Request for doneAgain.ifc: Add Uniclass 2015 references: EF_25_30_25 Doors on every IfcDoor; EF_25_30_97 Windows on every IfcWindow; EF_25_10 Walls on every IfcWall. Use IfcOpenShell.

First a look at what the model holds.

```python
import ifcopenshell

model = ifcopenshell.open("doneAgain.ifc")
print(model.schema)
print("classifications:", [c.Name for c in model.by_type("IfcClassification")])
for ifc_class in ("IfcDoor", "IfcRoof", "IfcStair", "IfcWall", "IfcWindow"):
    print(ifc_class, len(model.by_type(ifc_class)))
```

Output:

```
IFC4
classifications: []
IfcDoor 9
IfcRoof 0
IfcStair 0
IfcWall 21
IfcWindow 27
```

```python
import ifcopenshell
import ifcopenshell.api.classification

model = ifcopenshell.open("doneAgain.ifc")

system = ifcopenshell.api.classification.add_classification(model, classification="Uniclass 2015")

codes = {
    "IfcDoor": ("EF_25_30_25", "Doors"),
    "IfcWindow": ("EF_25_30_97", "Windows"),
    "IfcWall": ("EF_25_10", "Walls"),
}
for ifc_class, (code, name) in codes.items():
    products = model.by_type(ifc_class)
    ifcopenshell.api.classification.add_reference(
        model, products=products, classification=system, identification=code, name=name
    )
    print(code, len(products))

model.write("doneAgain_rev.ifc")
```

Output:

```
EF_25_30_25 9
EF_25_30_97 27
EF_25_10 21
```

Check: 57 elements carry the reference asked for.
